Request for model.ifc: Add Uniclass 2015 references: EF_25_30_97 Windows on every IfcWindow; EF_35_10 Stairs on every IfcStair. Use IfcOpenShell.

First a look at what the model holds.

```python
import ifcopenshell

model = ifcopenshell.open("model.ifc")
print(model.schema)
print("classifications:", [c.Name for c in model.by_type("IfcClassification")])
for ifc_class in ("IfcDoor", "IfcRoof", "IfcStair", "IfcWall", "IfcWindow"):
    print(ifc_class, len(model.by_type(ifc_class)))
```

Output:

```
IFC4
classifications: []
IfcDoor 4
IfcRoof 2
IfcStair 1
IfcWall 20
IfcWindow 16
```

```python
import ifcopenshell
import ifcopenshell.api.classification

model = ifcopenshell.open("model.ifc")

system = ifcopenshell.api.classification.add_classification(model, classification="Uniclass 2015")

codes = {
    "IfcWindow": ("EF_25_30_97", "Windows"),
    "IfcStair": ("EF_35_10", "Stairs"),
}
for ifc_class, (code, name) in codes.items():
    products = model.by_type(ifc_class)
    ifcopenshell.api.classification.add_reference(
        model, products=products, classification=system, identification=code, name=name
    )
    print(code, len(products))

model.write("model_updated.ifc")
```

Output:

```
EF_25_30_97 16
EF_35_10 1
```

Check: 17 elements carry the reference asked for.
